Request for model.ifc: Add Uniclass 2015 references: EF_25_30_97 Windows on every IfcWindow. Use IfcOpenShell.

First a look at what the model holds.

```python
import ifcopenshell

model = ifcopenshell.open("model.ifc")
print(model.schema)
print("classifications:", [c.Name for c in model.by_type("IfcClassification")])
for ifc_class in ("IfcDoor", "IfcRoof", "IfcStair", "IfcWall", "IfcWindow"):
    print(ifc_class, len(model.by_type(ifc_class)))
```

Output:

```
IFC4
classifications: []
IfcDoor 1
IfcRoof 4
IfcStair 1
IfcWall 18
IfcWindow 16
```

```python
import ifcopenshell
import ifcopenshell.api.classification

model = ifcopenshell.open("model.ifc")

system = ifcopenshell.api.classification.add_classification(model, classification="Uniclass 2015")

codes = {
    "IfcWindow": ("EF_25_30_97", "Windows"),
}
for ifc_class, (code, name) in codes.items():
    products = model.by_type(ifc_class)
    ifcopenshell.api.classification.add_reference(
        model, products=products, classification=system, identification=code, name=name
    )
    print(code, len(products))

model.write("model_edited.ifc")
```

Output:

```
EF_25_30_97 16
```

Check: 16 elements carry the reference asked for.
